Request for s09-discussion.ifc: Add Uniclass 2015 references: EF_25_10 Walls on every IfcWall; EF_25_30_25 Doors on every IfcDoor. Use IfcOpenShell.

First a look at what the model holds.

```python
import ifcopenshell

model = ifcopenshell.open("s09-discussion.ifc")
print(model.schema)
print("classifications:", [c.Name for c in model.by_type("IfcClassification")])
for ifc_class in ("IfcDoor", "IfcRoof", "IfcStair", "IfcWall", "IfcWindow"):
    print(ifc_class, len(model.by_type(ifc_class)))
```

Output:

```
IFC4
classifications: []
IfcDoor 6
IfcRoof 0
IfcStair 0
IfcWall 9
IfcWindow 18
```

```python
import ifcopenshell
import ifcopenshell.api.classification

model = ifcopenshell.open("s09-discussion.ifc")

system = ifcopenshell.api.classification.add_classification(model, classification="Uniclass 2015")

codes = {
    "IfcWall": ("EF_25_10", "Walls"),
    "IfcDoor": ("EF_25_30_25", "Doors"),
}
for ifc_class, (code, name) in codes.items():
    products = model.by_type(ifc_class)
    ifcopenshell.api.classification.add_reference(
        model, products=products, classification=system, identification=code, name=name
    )
    print(code, len(products))

model.write("s09-discussion_v2.ifc")
```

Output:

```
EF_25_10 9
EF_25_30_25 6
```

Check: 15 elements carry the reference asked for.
